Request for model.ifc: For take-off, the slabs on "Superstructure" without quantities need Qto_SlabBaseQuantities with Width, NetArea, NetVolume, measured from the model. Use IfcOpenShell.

First a look at what the model holds.

```python
import ifcopenshell
import ifcopenshell.util.element
import ifcopenshell.util.unit

model = ifcopenshell.open("model.ifc")
print(model.schema)
for unit_type in ("LENGTHUNIT", "AREAUNIT", "VOLUMEUNIT"):
    print(unit_type, ifcopenshell.util.unit.calculate_unit_scale(model, unit_type))
storey = next(s for s in model.by_type("IfcBuildingStorey") if s.Name == "Superstructure")
slabs = [e for e in ifcopenshell.util.element.get_decomposition(storey) if e.is_a("IfcSlab")]
for e in sorted(slabs, key=lambda e: e.id()):
    print(e.id(), e.is_a(), e.Name, list(ifcopenshell.util.element.get_psets(e, qtos_only=True)), sep=" | ")
```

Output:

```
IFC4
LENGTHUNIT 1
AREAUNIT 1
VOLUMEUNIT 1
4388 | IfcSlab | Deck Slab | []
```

```python
import ifcopenshell
import ifcopenshell.api.pset
import ifcopenshell.geom
import ifcopenshell.util.element
import ifcopenshell.util.shape
import ifcopenshell.util.unit

model = ifcopenshell.open("model.ifc")
unit_scale = ifcopenshell.util.unit.calculate_unit_scale(model)
area_scale = ifcopenshell.util.unit.calculate_unit_scale(model, "AREAUNIT")
volume_scale = ifcopenshell.util.unit.calculate_unit_scale(model, "VOLUMEUNIT")
settings = ifcopenshell.geom.settings()

storey = next(s for s in model.by_type("IfcBuildingStorey") if s.Name == "Superstructure")
slabs = [e for e in ifcopenshell.util.element.get_decomposition(storey) if e.is_a("IfcSlab")]

for e in sorted(slabs, key=lambda e: e.id()):
    if ifcopenshell.util.element.get_psets(e, qtos_only=True, should_inherit=False):
        continue
    # Geometry comes back in metres, in the element's own axes.
    shape = ifcopenshell.geom.create_shape(settings, e)
    values = {
        "Width": ifcopenshell.util.shape.get_z(shape.geometry) / unit_scale,
        "NetArea": ifcopenshell.util.shape.get_footprint_area(shape.geometry) / area_scale,
        "NetVolume": ifcopenshell.util.shape.get_volume(shape.geometry) / volume_scale,
    }
    qto = ifcopenshell.api.pset.add_qto(model, product=e, name="Qto_SlabBaseQuantities")
    ifcopenshell.api.pset.edit_qto(model, qto=qto, properties=values)
    print(e.id(), {k: round(v, 3) for k, v in values.items()})

model.write("model-out.ifc")
```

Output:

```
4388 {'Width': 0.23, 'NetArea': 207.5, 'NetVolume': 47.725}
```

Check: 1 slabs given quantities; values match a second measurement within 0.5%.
